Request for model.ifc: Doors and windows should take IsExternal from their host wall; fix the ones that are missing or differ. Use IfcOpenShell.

First a look at what the model holds.

```python
import ifcopenshell
import ifcopenshell.util.element

model = ifcopenshell.open("model.ifc")
print(model.schema)
seen = {}
for e in model.by_type("IfcDoor") + model.by_type("IfcWindow"):
    if not e.FillsVoids:
        continue
    host = e.FillsVoids[0].RelatingOpeningElement.VoidsElements[0].RelatingBuildingElement
    own = ifcopenshell.util.element.get_pset(e, f"Pset_{e.is_a()[3:].removesuffix('StandardCase')}Common", "IsExternal")
    wall = ifcopenshell.util.element.get_pset(host, "Pset_WallCommon", "IsExternal")
    seen[e.is_a(), own, wall] = seen.get((e.is_a(), own, wall), 0) + 1
for (cls, own, wall), count in sorted(seen.items(), key=str):
    print(count, cls, "IsExternal:", own, "| host wall:", wall)
```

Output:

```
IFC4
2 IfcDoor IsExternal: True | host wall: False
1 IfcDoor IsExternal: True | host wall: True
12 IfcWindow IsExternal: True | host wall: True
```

```python
import ifcopenshell
import ifcopenshell.api.pset
import ifcopenshell.util.element

model = ifcopenshell.open("model.ifc")

count = 0
for ifc_class, pset_name in (("IfcDoor", "Pset_DoorCommon"), ("IfcWindow", "Pset_WindowCommon")):
    for e in model.by_type(ifc_class):
        if not e.FillsVoids:
            continue
        host = e.FillsVoids[0].RelatingOpeningElement.VoidsElements[0].RelatingBuildingElement
        external = ifcopenshell.util.element.get_pset(host, "Pset_WallCommon", "IsExternal")
        if external is None or ifcopenshell.util.element.get_pset(e, pset_name, "IsExternal") == external:
            continue
        pset = ifcopenshell.api.pset.add_pset(model, product=e, name=pset_name)
        ifcopenshell.api.pset.edit_pset(model, pset=pset, properties={"IsExternal": external})
        count += 1

print(count, "updated")

model.write("model_edited.ifc")
```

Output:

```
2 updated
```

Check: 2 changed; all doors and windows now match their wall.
